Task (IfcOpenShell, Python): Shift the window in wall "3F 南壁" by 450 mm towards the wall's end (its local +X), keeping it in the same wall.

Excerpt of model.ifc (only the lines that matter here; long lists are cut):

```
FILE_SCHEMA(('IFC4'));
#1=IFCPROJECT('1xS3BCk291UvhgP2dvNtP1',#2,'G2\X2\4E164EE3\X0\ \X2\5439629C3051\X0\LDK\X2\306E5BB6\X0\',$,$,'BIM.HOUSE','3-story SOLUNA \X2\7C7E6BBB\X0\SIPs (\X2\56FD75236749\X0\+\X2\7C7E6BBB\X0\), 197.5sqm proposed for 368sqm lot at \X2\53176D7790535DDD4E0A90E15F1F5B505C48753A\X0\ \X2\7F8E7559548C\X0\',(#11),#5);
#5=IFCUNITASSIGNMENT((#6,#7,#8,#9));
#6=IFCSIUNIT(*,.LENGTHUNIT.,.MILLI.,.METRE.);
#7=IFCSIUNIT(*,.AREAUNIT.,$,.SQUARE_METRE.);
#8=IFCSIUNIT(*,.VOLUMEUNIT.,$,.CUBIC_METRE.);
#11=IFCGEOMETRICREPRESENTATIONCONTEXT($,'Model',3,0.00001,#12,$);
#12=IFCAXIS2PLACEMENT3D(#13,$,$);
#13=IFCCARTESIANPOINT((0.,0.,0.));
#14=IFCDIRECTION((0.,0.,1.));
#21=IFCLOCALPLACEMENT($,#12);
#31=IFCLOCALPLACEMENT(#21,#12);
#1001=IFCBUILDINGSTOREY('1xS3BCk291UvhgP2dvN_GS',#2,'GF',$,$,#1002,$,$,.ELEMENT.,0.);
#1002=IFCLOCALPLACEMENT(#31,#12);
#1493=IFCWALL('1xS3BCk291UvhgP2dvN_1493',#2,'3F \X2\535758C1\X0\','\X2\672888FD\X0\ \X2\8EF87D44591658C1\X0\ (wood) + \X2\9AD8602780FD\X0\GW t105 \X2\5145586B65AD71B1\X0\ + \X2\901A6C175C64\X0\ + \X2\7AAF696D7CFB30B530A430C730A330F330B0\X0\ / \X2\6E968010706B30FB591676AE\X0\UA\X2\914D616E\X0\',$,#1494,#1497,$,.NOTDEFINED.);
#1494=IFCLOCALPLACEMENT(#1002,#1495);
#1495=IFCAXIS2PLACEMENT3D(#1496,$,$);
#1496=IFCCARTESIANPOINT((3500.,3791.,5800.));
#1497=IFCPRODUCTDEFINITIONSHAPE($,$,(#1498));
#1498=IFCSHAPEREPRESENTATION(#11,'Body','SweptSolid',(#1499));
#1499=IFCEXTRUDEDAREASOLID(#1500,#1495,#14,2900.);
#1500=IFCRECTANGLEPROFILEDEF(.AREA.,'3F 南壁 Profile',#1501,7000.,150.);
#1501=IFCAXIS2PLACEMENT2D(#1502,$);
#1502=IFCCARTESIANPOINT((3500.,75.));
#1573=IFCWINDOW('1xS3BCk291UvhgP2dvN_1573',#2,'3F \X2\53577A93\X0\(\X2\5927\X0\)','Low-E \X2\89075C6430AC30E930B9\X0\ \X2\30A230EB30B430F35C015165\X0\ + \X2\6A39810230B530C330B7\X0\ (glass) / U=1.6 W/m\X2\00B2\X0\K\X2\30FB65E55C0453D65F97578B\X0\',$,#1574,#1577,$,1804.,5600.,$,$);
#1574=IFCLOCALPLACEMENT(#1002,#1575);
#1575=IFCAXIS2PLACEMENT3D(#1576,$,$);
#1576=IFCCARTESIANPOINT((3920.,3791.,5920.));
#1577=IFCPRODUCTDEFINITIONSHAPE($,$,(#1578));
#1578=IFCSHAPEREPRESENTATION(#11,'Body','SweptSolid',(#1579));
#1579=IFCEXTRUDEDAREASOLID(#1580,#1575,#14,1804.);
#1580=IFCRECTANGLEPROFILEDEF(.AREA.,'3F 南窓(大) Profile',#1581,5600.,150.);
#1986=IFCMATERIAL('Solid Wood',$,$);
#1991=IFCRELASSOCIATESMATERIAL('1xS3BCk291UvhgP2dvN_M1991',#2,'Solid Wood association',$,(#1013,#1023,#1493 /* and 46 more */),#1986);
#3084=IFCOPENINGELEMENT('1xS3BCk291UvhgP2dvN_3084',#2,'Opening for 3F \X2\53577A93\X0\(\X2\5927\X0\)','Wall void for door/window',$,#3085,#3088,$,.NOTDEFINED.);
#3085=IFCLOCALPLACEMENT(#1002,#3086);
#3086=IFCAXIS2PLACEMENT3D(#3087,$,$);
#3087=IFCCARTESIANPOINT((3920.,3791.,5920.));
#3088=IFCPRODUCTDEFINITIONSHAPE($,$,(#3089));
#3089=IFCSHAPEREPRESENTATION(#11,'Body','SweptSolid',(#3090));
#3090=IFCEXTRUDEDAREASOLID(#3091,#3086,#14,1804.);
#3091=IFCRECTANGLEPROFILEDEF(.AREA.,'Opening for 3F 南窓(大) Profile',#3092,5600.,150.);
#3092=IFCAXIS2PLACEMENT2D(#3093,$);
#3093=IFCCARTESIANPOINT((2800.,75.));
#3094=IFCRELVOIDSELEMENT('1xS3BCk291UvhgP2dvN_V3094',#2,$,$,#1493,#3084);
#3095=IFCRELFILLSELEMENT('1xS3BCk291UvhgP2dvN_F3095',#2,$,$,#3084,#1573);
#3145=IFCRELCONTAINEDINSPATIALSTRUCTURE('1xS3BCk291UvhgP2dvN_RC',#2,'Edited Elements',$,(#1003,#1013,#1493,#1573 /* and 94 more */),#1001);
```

```python
import ifcopenshell
import ifcopenshell.api.geometry
import ifcopenshell.util.placement
import ifcopenshell.util.unit

model = ifcopenshell.open("model.ifc")
unit_scale = ifcopenshell.util.unit.calculate_unit_scale(model)

window = model.by_id(1573)
opening = window.FillsVoids[0].RelatingOpeningElement
wall = opening.VoidsElements[0].RelatingBuildingElement

wall_matrix = ifcopenshell.util.placement.get_local_placement(wall.ObjectPlacement)
shift = wall_matrix[:3, 0] * 0.45 / unit_scale
before = ifcopenshell.util.placement.get_local_placement(window.ObjectPlacement)[:3, 3].copy()

# The window is not placed relative to its opening, so move both.
for product in (opening, window):
    matrix = ifcopenshell.util.placement.get_local_placement(product.ObjectPlacement)
    matrix[:3, 3] += shift
    ifcopenshell.api.geometry.edit_object_placement(model, product=product, matrix=matrix, is_si=False)

after = ifcopenshell.util.placement.get_local_placement(window.ObjectPlacement)[:3, 3]
print("window moved by", (after - before).round(3) + 0.0)

model.write("model_v2.ifc")
```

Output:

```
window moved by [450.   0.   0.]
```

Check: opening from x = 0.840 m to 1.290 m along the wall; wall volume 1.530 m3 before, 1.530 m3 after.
